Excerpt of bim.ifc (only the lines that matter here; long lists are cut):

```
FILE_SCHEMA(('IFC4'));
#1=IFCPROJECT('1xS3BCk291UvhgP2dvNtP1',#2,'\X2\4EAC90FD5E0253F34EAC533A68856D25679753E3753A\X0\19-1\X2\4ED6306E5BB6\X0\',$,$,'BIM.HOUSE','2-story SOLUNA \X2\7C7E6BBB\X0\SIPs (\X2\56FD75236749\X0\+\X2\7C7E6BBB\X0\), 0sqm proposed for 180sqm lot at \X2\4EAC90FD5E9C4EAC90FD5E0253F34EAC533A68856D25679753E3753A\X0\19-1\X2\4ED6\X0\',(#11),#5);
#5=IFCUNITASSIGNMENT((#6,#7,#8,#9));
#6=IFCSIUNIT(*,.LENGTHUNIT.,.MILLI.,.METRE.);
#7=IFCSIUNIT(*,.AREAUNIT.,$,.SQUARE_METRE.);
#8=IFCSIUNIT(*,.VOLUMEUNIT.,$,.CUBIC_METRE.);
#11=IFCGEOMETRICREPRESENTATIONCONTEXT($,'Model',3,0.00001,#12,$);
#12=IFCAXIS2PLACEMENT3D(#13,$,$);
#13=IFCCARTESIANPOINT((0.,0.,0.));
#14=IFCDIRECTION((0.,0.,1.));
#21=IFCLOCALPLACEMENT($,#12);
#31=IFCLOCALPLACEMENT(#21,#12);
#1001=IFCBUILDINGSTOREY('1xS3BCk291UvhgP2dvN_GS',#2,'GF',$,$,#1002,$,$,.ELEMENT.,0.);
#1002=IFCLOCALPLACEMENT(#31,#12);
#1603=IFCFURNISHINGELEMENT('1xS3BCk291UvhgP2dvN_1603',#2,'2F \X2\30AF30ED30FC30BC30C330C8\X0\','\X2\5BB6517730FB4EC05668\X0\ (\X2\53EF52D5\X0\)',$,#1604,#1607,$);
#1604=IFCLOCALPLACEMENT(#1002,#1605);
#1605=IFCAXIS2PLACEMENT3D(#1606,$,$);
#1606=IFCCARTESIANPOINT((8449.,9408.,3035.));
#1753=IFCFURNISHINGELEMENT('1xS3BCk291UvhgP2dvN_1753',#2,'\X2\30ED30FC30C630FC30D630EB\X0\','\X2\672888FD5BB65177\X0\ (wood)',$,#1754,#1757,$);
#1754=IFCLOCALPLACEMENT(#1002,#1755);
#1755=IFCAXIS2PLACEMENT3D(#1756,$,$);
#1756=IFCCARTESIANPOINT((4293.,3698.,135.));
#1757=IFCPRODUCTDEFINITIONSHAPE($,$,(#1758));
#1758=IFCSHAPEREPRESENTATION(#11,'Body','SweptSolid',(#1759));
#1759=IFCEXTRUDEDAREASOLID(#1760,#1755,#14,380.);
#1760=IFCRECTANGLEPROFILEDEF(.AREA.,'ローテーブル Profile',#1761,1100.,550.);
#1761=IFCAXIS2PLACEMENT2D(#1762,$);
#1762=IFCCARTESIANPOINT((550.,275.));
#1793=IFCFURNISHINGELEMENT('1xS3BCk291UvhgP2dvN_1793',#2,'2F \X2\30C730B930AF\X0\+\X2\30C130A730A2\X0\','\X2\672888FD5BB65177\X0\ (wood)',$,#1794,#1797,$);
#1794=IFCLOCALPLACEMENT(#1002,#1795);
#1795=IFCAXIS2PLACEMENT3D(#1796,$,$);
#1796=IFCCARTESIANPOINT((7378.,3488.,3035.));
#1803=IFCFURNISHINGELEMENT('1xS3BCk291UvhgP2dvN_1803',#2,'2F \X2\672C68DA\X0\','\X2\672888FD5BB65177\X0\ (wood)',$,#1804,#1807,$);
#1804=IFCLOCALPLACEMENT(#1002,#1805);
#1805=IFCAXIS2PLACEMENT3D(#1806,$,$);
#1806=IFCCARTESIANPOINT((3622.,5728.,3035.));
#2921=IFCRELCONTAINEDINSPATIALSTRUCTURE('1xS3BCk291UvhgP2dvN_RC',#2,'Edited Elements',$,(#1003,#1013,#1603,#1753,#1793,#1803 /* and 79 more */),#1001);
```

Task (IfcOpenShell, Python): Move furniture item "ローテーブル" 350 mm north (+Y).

```python
import ifcopenshell
import ifcopenshell.api.geometry
import ifcopenshell.util.placement
import ifcopenshell.util.unit

model = ifcopenshell.open("bim.ifc")
unit_scale = ifcopenshell.util.unit.calculate_unit_scale(model)

item = model.by_id(1753)
matrix = ifcopenshell.util.placement.get_local_placement(item.ObjectPlacement)
matrix[1, 3] += 0.35 / unit_scale
ifcopenshell.api.geometry.edit_object_placement(model, product=item, matrix=matrix, is_si=False)

print(ifcopenshell.util.placement.get_local_placement(item.ObjectPlacement).round(3) + 0.0)

model.write("bim_edited.ifc")
```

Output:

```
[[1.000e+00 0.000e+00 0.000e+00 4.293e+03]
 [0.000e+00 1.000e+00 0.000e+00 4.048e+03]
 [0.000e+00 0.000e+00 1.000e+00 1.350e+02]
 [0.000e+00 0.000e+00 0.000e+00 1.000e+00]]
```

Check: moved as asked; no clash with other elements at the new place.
